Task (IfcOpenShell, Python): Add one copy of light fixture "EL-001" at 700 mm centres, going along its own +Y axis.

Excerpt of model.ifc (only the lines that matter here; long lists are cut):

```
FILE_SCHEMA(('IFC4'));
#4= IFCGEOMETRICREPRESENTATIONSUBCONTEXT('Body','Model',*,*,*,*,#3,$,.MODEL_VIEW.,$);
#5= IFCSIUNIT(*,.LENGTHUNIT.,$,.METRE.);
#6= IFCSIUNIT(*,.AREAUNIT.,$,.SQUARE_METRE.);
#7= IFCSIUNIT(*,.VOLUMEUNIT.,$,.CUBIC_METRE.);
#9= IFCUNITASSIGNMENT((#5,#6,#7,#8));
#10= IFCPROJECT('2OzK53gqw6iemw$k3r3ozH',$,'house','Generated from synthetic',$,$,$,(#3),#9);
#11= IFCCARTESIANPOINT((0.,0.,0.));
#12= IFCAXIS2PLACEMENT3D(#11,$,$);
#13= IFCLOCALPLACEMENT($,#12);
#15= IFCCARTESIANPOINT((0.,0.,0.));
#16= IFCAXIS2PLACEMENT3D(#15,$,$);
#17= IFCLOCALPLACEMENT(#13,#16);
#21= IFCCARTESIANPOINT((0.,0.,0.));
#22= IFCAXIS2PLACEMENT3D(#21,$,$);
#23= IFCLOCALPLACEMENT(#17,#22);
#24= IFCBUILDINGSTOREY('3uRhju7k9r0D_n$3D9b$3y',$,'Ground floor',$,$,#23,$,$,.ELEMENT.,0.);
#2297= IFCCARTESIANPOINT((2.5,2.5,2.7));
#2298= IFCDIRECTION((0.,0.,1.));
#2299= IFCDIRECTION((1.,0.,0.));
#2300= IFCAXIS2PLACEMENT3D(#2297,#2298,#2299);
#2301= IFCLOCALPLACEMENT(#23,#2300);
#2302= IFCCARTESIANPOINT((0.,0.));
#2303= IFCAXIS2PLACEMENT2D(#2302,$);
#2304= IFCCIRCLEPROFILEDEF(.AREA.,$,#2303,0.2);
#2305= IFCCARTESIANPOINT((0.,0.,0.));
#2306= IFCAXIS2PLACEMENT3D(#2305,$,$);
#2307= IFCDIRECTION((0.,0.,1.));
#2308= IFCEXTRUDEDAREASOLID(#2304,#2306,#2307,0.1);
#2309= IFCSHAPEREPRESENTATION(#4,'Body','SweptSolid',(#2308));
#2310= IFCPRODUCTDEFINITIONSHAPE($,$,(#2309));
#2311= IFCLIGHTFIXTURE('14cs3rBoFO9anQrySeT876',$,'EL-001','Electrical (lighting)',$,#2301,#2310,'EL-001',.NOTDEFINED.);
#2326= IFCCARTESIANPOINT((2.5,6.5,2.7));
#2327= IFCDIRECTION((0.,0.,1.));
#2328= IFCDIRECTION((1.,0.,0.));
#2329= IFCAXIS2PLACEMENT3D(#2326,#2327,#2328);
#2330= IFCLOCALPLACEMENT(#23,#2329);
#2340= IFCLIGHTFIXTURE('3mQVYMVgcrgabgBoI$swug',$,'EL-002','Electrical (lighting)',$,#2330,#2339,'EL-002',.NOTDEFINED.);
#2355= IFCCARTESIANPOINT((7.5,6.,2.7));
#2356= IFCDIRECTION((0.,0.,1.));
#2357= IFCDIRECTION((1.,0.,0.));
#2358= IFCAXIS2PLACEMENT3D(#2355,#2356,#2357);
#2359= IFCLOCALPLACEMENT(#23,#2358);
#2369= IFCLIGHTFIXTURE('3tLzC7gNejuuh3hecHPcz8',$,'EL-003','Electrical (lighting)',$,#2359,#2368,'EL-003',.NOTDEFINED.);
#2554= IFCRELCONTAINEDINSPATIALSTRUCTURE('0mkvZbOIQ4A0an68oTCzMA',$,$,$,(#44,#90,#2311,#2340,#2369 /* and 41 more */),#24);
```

```python
import ifcopenshell
import ifcopenshell.api.geometry
import ifcopenshell.api.root
import ifcopenshell.util.element
import ifcopenshell.util.placement

model = ifcopenshell.open("model.ifc")

source = model.by_guid("14cs3rBoFO9anQrySeT876")
base = ifcopenshell.util.placement.get_local_placement(source.ObjectPlacement)
step = base[:3, 1] * 0.7

for i in range(1, 2):
    copy = ifcopenshell.api.root.copy_class(model, product=source)
    copy.Representation = ifcopenshell.util.element.copy_deep(
        model, source.Representation, exclude=["IfcGeometricRepresentationContext", "IfcRepresentationMap"]
    )
    copy.Tag = None
    matrix = base.copy()
    matrix[:3, 3] += i * step
    print("added at", matrix[:3, 3].round(3) + 0.0)
    ifcopenshell.api.geometry.edit_object_placement(model, product=copy, matrix=matrix, is_si=False)

model.write("model-out.ifc")
```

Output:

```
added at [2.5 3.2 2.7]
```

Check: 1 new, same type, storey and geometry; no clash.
